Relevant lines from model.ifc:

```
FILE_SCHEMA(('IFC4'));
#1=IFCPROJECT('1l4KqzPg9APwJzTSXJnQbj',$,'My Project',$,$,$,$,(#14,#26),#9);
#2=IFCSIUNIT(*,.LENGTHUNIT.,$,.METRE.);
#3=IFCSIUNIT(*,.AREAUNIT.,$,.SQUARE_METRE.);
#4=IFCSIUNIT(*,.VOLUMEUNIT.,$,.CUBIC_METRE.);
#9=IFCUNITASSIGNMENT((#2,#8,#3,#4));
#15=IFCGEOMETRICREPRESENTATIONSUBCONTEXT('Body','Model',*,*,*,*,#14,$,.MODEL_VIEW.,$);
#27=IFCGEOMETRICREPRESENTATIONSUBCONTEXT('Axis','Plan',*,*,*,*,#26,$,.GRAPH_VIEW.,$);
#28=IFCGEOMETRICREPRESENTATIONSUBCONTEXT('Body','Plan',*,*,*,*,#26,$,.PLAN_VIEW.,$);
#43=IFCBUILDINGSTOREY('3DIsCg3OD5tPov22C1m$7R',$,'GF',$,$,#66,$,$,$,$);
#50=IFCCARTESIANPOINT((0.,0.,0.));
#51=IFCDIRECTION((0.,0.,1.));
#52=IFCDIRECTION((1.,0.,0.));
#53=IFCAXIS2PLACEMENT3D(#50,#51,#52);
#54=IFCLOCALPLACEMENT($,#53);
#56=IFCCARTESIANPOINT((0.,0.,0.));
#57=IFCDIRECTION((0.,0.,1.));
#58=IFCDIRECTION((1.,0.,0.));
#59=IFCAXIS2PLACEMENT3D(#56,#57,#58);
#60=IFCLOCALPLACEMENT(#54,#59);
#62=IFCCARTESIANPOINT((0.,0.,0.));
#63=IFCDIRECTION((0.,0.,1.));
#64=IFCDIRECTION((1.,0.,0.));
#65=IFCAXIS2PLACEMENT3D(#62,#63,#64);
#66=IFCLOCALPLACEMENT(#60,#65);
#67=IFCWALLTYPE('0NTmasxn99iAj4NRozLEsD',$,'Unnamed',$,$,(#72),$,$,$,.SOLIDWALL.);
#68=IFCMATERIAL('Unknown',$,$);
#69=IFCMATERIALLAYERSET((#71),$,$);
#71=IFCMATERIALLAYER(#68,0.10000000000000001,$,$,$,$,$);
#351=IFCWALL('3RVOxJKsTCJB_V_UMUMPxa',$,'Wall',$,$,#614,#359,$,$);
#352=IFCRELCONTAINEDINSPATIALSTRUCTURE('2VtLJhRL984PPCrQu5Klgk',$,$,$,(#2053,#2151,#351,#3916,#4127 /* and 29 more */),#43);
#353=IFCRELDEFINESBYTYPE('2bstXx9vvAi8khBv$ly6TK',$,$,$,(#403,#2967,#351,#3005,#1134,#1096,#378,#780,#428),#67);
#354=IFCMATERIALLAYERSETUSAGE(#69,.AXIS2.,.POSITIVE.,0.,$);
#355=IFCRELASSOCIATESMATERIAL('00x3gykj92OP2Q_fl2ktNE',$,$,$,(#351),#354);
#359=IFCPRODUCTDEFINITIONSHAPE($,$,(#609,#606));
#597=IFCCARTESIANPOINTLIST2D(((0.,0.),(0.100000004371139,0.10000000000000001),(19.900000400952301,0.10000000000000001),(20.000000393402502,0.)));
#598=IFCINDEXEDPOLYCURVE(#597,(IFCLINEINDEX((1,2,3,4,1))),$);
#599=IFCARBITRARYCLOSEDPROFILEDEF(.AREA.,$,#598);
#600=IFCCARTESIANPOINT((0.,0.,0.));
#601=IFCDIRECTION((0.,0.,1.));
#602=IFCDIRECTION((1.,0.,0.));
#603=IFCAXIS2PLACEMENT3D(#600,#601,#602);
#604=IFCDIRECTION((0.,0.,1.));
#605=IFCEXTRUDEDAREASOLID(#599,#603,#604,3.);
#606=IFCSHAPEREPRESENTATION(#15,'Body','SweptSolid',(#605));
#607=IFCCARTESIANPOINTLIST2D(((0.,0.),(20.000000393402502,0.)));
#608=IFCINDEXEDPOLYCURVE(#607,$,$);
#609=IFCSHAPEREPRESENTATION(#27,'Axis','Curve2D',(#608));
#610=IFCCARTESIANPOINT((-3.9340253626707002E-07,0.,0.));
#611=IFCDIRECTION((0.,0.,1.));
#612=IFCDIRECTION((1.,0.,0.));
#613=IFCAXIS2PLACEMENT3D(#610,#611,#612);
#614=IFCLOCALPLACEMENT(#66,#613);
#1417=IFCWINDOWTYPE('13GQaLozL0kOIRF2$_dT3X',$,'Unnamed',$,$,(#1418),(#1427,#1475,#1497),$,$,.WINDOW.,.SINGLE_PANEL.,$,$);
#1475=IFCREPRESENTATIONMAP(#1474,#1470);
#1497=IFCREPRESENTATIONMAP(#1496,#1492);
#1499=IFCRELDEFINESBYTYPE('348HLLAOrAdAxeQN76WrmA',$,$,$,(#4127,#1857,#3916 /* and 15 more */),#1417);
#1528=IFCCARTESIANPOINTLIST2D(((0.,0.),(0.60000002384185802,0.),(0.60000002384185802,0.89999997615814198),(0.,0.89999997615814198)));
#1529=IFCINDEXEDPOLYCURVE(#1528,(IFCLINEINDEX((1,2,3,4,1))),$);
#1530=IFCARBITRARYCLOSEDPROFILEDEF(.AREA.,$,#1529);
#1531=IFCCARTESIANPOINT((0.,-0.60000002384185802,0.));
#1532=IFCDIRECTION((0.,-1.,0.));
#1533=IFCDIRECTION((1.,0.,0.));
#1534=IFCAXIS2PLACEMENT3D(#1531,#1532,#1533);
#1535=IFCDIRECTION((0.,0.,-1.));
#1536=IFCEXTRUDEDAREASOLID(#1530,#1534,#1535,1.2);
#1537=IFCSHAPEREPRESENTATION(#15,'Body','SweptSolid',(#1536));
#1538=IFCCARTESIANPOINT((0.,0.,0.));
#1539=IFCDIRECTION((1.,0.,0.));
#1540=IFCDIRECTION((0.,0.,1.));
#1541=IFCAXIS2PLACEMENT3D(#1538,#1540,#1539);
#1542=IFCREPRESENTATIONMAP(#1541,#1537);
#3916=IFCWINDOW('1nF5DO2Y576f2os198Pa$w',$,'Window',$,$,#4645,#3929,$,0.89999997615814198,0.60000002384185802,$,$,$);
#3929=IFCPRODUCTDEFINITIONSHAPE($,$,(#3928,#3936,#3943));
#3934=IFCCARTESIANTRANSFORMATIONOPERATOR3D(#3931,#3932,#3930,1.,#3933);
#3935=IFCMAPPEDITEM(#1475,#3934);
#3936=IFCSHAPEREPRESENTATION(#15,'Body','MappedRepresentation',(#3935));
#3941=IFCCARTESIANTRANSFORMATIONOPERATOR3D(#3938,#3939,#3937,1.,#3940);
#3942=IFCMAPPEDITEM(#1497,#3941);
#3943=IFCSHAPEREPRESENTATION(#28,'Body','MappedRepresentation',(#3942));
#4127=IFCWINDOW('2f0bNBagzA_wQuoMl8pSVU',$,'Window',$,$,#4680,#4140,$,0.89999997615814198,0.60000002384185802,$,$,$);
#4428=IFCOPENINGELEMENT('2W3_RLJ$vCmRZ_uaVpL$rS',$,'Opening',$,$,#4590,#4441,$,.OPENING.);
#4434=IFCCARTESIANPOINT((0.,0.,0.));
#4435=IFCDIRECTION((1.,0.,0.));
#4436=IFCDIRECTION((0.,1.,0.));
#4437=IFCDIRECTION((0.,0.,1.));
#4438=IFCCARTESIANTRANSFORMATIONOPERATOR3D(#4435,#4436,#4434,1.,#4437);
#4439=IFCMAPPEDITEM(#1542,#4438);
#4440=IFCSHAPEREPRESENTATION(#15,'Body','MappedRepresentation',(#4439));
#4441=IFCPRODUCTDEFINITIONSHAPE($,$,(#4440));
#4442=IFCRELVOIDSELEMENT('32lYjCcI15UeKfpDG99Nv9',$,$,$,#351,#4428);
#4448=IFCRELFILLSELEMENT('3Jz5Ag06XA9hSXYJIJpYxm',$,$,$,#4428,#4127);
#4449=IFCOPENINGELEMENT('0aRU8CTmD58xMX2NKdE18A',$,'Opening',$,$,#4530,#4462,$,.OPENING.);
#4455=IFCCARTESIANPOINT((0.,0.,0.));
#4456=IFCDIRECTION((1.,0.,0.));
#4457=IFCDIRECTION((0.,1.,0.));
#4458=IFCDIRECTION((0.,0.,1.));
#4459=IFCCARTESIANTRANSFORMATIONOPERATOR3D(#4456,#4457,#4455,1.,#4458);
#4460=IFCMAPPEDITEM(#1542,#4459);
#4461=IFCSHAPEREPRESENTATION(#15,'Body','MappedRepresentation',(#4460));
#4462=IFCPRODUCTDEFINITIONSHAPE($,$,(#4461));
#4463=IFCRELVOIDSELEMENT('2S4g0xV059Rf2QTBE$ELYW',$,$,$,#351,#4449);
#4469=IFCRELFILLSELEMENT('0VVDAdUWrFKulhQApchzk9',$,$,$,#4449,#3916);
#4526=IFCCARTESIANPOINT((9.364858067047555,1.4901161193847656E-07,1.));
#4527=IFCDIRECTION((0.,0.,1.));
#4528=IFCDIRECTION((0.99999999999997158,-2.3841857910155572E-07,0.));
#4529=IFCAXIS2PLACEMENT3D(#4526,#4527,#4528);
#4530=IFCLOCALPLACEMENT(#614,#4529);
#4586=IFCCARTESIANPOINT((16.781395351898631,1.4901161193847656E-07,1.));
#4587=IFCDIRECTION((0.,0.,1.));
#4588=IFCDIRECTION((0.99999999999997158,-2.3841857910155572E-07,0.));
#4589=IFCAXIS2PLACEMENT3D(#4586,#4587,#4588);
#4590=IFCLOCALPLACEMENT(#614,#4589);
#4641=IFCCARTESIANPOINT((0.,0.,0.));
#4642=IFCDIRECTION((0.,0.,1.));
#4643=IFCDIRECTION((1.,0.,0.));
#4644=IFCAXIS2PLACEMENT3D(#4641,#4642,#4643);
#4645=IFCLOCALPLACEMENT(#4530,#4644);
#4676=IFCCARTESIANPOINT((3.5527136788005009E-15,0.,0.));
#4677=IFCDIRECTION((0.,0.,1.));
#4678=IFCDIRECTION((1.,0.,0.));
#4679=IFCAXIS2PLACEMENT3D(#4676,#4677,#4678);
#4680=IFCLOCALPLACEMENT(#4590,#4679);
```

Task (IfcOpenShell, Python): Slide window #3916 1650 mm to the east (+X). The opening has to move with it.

```python
import ifcopenshell
import ifcopenshell.api.geometry
import ifcopenshell.util.placement
import ifcopenshell.util.unit

model = ifcopenshell.open("model.ifc")
unit_scale = ifcopenshell.util.unit.calculate_unit_scale(model)

window = model.by_guid("1nF5DO2Y576f2os198Pa$w")
opening = window.FillsVoids[0].RelatingOpeningElement
wall = opening.VoidsElements[0].RelatingBuildingElement

wall_matrix = ifcopenshell.util.placement.get_local_placement(wall.ObjectPlacement)
shift = wall_matrix[:3, 0] * 1.65 / unit_scale
before = ifcopenshell.util.placement.get_local_placement(window.ObjectPlacement)[:3, 3].copy()

# The window is placed relative to its opening, so it follows when the opening moves.
matrix = ifcopenshell.util.placement.get_local_placement(opening.ObjectPlacement)
matrix[:3, 3] += shift
ifcopenshell.api.geometry.edit_object_placement(
    model, product=opening, matrix=matrix, is_si=False, should_transform_children=True
)

after = ifcopenshell.util.placement.get_local_placement(window.ObjectPlacement)[:3, 3]
print("window moved by", (after - before).round(3) + 0.0)

model.write("model_v2.ifc")
```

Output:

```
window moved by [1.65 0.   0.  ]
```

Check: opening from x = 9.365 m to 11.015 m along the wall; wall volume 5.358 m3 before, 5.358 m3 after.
